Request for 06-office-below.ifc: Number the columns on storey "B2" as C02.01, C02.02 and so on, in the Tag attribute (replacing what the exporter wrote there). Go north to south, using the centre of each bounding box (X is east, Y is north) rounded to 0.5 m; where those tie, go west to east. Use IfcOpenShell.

First a look at what the model holds.

```python
import ifcopenshell
import ifcopenshell.util.element
import ifcopenshell.util.placement

model = ifcopenshell.open("06-office-below.ifc")
print(model.schema)
storey = next(s for s in model.by_type("IfcBuildingStorey") if s.Name == "B2")
columns = [e for e in ifcopenshell.util.element.get_decomposition(storey) if e.is_a("IfcColumn")]
for e in sorted(columns, key=lambda e: e.id()):
    origin = ifcopenshell.util.placement.get_local_placement(e.ObjectPlacement)[:3, 3]
    print(e.id(), e.Tag, e.Name, origin.round(2) + 0.0, sep=" | ")
```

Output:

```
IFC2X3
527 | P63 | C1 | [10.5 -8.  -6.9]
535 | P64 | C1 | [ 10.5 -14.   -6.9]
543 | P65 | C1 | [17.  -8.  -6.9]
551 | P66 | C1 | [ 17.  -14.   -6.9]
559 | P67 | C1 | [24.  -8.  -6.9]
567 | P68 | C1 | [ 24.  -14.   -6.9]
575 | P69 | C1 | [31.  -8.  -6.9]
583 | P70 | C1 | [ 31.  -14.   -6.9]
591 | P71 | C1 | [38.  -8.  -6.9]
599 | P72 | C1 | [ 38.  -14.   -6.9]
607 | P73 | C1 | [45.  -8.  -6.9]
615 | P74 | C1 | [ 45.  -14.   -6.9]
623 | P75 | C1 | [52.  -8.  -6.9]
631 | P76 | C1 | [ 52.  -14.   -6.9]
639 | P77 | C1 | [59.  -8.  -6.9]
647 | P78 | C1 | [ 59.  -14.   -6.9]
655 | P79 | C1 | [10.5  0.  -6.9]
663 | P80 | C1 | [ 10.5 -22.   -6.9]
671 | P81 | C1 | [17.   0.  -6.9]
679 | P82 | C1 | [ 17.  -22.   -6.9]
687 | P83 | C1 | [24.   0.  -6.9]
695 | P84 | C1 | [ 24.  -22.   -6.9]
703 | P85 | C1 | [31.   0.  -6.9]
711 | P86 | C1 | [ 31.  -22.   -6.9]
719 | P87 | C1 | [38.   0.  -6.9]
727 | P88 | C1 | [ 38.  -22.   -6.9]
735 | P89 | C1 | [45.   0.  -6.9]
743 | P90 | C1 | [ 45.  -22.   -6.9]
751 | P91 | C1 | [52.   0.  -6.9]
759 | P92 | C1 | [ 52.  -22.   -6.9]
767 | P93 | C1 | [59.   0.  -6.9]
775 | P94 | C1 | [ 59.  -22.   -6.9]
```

```python
import ifcopenshell
import ifcopenshell.geom
import ifcopenshell.util.element
import ifcopenshell.util.shape

model = ifcopenshell.open("06-office-below.ifc")
settings = ifcopenshell.geom.settings()
settings.set("use-world-coords", True)


def centre(element):
    shape = ifcopenshell.geom.create_shape(settings, element)
    return ifcopenshell.util.shape.get_bbox_centroid(shape.geometry)


storey = next(s for s in model.by_type("IfcBuildingStorey") if s.Name == "B2")
columns = [e for e in ifcopenshell.util.element.get_decomposition(storey) if e.is_a("IfcColumn")]

# Insertion points can sit at a corner or the storey origin, so sort by the geometry (in metres).
centres = {e: centre(e) for e in columns}
columns.sort(key=lambda e: (-round(centres[e][1] / 0.5), centres[e][0]))

for i, e in enumerate(columns, start=1):
    number = f"C02.{i:02d}"
    e.Tag = number
    print(e.id(), number)

model.write("06-office-below_updated.ifc")
```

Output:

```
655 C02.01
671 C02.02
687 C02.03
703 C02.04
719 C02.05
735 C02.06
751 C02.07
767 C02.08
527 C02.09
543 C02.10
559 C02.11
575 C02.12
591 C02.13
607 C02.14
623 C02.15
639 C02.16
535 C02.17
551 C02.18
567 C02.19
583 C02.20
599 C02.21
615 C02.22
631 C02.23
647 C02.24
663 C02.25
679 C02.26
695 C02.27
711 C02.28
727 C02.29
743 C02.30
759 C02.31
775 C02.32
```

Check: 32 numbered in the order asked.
